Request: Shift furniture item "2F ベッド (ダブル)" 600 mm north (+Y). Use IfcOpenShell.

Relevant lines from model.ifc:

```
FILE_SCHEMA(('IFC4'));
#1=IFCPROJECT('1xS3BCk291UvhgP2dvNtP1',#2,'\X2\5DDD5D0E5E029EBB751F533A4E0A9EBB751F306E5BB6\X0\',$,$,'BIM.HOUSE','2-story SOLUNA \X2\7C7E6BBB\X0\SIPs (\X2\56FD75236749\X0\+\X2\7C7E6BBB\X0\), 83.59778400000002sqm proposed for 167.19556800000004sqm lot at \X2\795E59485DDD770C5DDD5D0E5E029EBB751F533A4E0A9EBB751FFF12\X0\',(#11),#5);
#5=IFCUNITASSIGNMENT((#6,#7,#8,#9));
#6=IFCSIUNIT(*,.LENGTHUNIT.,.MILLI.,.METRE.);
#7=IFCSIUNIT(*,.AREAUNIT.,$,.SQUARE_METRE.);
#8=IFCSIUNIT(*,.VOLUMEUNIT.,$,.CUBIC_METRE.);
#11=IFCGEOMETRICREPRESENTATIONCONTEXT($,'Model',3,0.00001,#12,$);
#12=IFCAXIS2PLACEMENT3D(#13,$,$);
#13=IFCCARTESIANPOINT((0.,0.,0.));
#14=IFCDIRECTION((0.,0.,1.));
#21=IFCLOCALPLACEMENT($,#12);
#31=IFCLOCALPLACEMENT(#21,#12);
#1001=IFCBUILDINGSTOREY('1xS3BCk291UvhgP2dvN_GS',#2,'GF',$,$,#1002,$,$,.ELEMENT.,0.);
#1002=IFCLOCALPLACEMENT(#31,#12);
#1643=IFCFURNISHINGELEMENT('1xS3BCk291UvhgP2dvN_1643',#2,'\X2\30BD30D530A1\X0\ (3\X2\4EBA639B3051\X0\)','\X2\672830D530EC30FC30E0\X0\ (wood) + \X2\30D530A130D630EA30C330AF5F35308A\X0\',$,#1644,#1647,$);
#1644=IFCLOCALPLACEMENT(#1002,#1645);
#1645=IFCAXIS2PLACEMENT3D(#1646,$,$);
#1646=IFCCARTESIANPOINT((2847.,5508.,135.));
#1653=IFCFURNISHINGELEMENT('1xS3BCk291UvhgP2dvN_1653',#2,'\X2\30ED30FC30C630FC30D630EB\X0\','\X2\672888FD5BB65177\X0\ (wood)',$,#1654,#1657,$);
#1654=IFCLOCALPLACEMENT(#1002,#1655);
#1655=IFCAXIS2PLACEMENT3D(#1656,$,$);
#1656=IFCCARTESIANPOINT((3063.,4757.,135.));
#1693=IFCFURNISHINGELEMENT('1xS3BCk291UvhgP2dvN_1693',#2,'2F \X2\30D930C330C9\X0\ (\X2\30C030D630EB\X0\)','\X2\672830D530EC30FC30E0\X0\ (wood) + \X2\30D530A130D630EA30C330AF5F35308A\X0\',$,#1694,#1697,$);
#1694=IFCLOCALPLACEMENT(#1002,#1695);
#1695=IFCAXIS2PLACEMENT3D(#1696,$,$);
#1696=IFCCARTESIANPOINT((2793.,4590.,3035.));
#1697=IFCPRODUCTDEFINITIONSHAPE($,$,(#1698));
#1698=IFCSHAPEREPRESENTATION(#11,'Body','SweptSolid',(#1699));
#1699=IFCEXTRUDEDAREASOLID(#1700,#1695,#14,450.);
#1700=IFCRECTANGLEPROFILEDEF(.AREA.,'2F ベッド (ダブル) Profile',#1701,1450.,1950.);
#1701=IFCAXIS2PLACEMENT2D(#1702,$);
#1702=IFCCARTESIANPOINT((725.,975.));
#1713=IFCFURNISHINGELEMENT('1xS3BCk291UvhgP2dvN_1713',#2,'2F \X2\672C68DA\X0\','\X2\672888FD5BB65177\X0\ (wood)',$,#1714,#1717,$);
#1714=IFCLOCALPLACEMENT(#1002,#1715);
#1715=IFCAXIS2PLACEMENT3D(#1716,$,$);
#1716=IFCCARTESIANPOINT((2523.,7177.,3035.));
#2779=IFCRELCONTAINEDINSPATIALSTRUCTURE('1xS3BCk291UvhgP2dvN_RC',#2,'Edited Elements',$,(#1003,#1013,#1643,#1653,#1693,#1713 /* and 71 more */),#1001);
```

```python
import ifcopenshell
import ifcopenshell.api.geometry
import ifcopenshell.util.placement

model = ifcopenshell.open("model.ifc")

item = model.by_id(1693)
matrix = ifcopenshell.util.placement.get_local_placement(item.ObjectPlacement)
matrix[1, 3] += 600.0
ifcopenshell.api.geometry.edit_object_placement(model, product=item, matrix=matrix, is_si=False)

print(ifcopenshell.util.placement.get_local_placement(item.ObjectPlacement).round(3) + 0.0)

model.write("model_v2.ifc")
```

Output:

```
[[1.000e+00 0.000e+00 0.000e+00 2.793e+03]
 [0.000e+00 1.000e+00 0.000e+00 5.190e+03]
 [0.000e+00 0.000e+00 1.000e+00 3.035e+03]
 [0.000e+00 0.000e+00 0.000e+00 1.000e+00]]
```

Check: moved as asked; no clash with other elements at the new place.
